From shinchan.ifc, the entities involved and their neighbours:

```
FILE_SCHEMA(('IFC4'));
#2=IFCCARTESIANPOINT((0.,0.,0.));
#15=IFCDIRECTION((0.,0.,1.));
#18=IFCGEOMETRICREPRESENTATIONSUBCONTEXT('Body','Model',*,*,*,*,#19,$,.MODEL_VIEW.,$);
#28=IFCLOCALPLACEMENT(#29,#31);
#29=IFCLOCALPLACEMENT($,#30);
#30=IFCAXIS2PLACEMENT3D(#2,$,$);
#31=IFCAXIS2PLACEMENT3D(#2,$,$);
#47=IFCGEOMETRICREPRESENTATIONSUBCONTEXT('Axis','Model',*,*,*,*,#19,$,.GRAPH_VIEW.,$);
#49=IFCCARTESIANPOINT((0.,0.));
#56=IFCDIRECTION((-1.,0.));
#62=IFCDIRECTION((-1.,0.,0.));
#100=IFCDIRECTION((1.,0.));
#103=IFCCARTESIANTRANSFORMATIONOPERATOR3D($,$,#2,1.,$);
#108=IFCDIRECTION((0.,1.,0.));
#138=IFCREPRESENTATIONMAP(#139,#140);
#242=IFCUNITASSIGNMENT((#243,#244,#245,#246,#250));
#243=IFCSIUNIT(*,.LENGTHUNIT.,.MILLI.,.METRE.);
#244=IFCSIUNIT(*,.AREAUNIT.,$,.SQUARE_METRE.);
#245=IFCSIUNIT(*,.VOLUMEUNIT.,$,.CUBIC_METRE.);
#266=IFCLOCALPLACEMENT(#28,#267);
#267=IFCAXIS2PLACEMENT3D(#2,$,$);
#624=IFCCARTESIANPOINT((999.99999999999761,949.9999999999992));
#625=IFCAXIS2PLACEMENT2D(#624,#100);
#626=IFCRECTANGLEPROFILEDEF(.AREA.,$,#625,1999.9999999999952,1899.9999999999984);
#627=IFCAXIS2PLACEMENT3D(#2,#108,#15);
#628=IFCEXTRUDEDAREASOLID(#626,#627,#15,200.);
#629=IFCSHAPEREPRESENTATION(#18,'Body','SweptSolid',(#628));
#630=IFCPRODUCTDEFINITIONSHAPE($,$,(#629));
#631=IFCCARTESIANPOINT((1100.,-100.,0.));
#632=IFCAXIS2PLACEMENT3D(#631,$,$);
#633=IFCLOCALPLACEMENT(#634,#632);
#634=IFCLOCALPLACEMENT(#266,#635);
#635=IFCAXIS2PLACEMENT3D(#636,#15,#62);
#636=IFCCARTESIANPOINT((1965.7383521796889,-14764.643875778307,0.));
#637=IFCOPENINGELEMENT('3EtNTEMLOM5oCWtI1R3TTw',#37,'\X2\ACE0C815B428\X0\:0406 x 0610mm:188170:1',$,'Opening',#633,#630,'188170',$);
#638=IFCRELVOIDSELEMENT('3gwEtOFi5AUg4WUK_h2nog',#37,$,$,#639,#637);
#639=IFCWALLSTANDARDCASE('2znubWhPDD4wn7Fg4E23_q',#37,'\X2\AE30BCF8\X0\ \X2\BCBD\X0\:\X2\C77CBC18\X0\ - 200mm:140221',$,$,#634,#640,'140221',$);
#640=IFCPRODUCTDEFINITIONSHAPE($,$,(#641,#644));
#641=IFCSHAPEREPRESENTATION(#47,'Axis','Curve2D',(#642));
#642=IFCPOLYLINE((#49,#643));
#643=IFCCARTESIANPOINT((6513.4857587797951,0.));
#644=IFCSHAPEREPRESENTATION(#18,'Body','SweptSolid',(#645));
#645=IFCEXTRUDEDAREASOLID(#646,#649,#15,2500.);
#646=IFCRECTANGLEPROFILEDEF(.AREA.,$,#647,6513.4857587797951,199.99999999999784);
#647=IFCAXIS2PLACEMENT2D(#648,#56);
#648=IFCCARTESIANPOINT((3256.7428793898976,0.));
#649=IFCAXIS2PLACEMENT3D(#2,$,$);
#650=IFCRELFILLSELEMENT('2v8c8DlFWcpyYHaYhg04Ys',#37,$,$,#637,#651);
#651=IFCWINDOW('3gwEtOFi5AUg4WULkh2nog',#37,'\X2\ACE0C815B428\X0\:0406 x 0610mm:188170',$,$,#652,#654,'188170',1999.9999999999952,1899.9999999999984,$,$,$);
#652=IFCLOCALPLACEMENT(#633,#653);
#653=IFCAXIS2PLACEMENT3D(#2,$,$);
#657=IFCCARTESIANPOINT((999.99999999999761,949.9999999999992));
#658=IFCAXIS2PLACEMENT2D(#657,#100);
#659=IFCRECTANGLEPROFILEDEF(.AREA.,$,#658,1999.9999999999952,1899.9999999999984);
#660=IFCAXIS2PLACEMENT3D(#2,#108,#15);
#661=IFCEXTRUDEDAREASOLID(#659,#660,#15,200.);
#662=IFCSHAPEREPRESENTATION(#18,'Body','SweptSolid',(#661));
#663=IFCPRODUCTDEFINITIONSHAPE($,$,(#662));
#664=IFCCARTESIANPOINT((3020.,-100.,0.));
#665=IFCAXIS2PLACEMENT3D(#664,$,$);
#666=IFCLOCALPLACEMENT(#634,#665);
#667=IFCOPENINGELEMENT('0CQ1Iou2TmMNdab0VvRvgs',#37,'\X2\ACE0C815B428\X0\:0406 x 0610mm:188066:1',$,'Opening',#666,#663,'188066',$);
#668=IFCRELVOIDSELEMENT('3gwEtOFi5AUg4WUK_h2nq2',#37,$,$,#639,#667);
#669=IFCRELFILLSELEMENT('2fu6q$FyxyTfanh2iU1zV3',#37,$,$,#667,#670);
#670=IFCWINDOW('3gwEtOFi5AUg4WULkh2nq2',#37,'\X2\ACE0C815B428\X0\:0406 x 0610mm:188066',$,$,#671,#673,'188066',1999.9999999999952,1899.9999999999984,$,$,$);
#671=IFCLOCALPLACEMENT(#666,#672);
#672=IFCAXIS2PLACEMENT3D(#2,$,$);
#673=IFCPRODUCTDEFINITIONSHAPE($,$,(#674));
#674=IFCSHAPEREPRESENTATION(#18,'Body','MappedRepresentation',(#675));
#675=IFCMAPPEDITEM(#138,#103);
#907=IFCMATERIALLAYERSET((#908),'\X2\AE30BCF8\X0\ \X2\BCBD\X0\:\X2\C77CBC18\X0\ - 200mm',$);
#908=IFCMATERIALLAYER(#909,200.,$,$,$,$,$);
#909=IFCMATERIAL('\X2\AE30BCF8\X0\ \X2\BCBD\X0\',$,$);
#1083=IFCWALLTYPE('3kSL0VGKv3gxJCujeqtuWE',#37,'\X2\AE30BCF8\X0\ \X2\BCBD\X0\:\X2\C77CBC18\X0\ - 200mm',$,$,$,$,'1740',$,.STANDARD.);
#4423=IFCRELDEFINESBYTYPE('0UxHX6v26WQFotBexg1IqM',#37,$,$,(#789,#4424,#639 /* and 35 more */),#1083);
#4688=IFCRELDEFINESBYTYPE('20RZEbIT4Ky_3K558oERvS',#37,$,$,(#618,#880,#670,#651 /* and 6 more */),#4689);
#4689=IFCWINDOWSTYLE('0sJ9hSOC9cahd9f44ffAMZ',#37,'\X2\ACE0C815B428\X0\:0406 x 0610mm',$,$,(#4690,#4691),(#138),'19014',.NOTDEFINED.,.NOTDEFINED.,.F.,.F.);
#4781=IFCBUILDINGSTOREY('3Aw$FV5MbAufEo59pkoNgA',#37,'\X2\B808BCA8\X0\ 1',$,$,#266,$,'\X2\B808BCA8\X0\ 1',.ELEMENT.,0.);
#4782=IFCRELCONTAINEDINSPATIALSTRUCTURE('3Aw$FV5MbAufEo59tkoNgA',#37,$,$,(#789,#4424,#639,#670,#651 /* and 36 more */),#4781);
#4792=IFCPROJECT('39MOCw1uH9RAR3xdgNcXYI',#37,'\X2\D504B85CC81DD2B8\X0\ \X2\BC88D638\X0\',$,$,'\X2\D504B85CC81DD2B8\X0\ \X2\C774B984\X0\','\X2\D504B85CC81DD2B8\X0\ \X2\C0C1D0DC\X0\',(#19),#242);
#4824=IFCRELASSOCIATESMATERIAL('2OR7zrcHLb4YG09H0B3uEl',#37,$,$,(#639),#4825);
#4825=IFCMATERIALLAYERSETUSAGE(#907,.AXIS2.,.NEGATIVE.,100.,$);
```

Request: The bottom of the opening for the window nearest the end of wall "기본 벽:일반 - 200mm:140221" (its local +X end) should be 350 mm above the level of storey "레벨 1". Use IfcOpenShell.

```python
import numpy as np
import ifcopenshell
import ifcopenshell.api.geometry
import ifcopenshell.geom
import ifcopenshell.util.element
import ifcopenshell.util.placement
import ifcopenshell.util.shape
import ifcopenshell.util.unit

model = ifcopenshell.open("shinchan.ifc")
unit_scale = ifcopenshell.util.unit.calculate_unit_scale(model)

window = model.by_id(670)
opening = window.FillsVoids[0].RelatingOpeningElement
storey = ifcopenshell.util.element.get_container(window, ifc_class="IfcBuildingStorey")
level = ifcopenshell.util.placement.get_local_placement(storey.ObjectPlacement)[2, 3]

# The opening's origin need not be at the sill, so measure its lowest point.
shape = ifcopenshell.geom.create_shape(ifcopenshell.geom.settings(), opening)
bottom = ifcopenshell.util.shape.get_shape_bottom_elevation(shape, shape.geometry) / unit_scale
dz = level + 0.35 / unit_scale - bottom

shift = np.array([0.0, 0.0, dz])
# The window is placed relative to its opening, so it follows when the opening moves.
matrix = ifcopenshell.util.placement.get_local_placement(opening.ObjectPlacement)
matrix[:3, 3] += shift
ifcopenshell.api.geometry.edit_object_placement(
    model, product=opening, matrix=matrix, is_si=False, should_transform_children=True
)

print(f"moved by {dz * unit_scale:+.3f} m")

model.write("shinchan_v2.ifc")
```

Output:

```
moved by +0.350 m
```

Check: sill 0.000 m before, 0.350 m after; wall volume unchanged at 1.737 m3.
